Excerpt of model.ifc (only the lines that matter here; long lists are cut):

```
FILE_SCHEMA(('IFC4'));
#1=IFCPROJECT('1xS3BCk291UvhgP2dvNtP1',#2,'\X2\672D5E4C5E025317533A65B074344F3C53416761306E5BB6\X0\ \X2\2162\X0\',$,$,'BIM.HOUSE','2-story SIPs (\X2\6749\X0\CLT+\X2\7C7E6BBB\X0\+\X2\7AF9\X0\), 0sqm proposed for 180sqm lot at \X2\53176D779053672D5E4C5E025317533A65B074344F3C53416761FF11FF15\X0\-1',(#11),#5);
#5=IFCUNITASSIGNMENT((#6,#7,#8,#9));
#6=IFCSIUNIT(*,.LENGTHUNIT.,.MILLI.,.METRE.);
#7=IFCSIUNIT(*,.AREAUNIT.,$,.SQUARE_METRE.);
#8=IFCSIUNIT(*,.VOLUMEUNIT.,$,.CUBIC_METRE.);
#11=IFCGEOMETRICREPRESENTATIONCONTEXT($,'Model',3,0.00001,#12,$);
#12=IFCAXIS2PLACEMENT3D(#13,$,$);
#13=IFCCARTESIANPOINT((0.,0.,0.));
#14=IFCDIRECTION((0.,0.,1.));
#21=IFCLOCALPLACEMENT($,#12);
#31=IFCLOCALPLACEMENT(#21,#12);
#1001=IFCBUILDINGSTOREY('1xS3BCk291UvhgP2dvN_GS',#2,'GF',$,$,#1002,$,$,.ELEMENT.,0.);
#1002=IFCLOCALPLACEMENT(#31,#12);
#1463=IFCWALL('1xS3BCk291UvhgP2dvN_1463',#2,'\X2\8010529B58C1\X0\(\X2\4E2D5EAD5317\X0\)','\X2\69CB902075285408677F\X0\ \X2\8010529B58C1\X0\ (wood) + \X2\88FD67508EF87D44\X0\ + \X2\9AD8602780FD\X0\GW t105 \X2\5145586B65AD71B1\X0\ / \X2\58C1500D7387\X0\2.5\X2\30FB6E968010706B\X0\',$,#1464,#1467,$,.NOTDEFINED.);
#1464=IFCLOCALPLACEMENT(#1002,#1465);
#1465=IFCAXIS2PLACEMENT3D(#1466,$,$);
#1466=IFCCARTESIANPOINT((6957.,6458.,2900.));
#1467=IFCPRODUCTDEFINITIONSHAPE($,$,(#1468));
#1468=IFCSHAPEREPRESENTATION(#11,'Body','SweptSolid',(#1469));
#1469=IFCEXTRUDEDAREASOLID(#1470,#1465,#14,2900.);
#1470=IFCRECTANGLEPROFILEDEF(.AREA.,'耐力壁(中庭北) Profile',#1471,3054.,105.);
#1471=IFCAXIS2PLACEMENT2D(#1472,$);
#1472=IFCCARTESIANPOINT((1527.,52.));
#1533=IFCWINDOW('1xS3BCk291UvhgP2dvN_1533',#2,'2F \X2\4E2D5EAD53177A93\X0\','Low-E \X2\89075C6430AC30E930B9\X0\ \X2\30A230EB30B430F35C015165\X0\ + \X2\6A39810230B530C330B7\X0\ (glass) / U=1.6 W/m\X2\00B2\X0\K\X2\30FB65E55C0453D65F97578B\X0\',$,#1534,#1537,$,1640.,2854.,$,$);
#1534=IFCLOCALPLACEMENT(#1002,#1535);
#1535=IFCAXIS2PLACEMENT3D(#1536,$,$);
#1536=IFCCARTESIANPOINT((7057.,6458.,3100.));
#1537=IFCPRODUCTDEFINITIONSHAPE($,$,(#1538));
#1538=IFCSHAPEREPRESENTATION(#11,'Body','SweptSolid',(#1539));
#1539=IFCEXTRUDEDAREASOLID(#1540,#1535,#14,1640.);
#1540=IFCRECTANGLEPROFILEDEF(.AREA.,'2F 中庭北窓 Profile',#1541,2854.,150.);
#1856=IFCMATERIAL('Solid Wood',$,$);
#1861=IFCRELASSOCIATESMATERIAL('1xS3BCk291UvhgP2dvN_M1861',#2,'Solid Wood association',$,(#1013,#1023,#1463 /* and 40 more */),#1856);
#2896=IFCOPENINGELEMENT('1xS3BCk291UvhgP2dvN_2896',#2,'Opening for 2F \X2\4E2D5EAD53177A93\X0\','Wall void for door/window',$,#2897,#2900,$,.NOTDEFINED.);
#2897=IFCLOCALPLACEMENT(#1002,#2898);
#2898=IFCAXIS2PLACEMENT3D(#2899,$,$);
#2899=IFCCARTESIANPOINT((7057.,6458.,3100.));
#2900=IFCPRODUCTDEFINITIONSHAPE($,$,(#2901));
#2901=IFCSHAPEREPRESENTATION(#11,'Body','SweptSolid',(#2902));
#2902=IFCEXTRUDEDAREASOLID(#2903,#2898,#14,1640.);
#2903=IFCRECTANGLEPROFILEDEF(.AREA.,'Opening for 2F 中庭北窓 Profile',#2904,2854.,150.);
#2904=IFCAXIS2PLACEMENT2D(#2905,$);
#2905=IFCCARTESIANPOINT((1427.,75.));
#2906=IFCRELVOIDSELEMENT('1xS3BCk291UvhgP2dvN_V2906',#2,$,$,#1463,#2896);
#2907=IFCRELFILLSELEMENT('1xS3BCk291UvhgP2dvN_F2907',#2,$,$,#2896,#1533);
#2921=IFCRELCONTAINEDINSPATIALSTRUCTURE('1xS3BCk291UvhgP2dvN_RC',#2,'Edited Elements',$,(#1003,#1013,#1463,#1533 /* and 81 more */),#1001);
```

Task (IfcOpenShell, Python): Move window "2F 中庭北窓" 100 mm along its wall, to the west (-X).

```python
import ifcopenshell
import ifcopenshell.api.geometry
import ifcopenshell.util.placement
import ifcopenshell.util.unit

model = ifcopenshell.open("model.ifc")
unit_scale = ifcopenshell.util.unit.calculate_unit_scale(model)

window = model.by_id(1533)
opening = window.FillsVoids[0].RelatingOpeningElement
wall = opening.VoidsElements[0].RelatingBuildingElement

wall_matrix = ifcopenshell.util.placement.get_local_placement(wall.ObjectPlacement)
shift = wall_matrix[:3, 0] * -0.1 / unit_scale
before = ifcopenshell.util.placement.get_local_placement(window.ObjectPlacement)[:3, 3].copy()

# The window is not placed relative to its opening, so move both.
for product in (opening, window):
    matrix = ifcopenshell.util.placement.get_local_placement(product.ObjectPlacement)
    matrix[:3, 3] += shift
    ifcopenshell.api.geometry.edit_object_placement(model, product=product, matrix=matrix, is_si=False)

after = ifcopenshell.util.placement.get_local_placement(window.ObjectPlacement)[:3, 3]
print("window moved by", (after - before).round(3) + 0.0)

model.write("model_rev.ifc")
```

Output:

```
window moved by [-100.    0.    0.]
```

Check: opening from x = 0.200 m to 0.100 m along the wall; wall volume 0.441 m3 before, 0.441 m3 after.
